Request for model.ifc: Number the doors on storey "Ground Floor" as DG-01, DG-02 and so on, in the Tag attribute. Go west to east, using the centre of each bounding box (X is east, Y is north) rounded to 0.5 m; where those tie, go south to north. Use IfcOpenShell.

First a look at what the model holds.

```python
import ifcopenshell
import ifcopenshell.util.element
import ifcopenshell.util.placement

model = ifcopenshell.open("model.ifc")
print(model.schema)
storey = next(s for s in model.by_type("IfcBuildingStorey") if s.Name == "Ground Floor")
doors = [e for e in ifcopenshell.util.element.get_decomposition(storey) if e.is_a("IfcDoor")]
for e in sorted(doors, key=lambda e: e.id()):
    origin = ifcopenshell.util.placement.get_local_placement(e.ObjectPlacement)[:3, 3]
    print(e.id(), e.Tag, e.Name, origin.round(2) + 0.0, sep=" | ")
```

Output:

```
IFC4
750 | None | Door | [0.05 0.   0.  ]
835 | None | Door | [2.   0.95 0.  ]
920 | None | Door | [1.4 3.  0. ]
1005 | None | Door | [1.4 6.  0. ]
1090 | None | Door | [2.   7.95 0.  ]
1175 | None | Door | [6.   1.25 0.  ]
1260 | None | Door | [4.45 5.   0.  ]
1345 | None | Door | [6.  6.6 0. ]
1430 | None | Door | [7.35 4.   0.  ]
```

```python
import ifcopenshell
import ifcopenshell.geom
import ifcopenshell.util.element
import ifcopenshell.util.shape

model = ifcopenshell.open("model.ifc")
settings = ifcopenshell.geom.settings()
settings.set("use-world-coords", True)


def centre(element):
    shape = ifcopenshell.geom.create_shape(settings, element)
    return ifcopenshell.util.shape.get_bbox_centroid(shape.geometry)


storey = next(s for s in model.by_type("IfcBuildingStorey") if s.Name == "Ground Floor")
doors = [e for e in ifcopenshell.util.element.get_decomposition(storey) if e.is_a("IfcDoor")]

# Insertion points can sit at a corner or the storey origin, so sort by the geometry (in metres).
centres = {e: centre(e) for e in doors}
doors.sort(key=lambda e: (round(centres[e][0] / 0.5), centres[e][1]))

for i, e in enumerate(doors, start=1):
    number = f"DG-{i:02d}"
    e.Tag = number
    print(e.id(), number)

model.write("model-out.ifc")
```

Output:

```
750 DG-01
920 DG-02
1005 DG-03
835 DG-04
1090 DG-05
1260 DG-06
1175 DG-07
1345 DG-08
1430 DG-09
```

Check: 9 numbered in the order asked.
